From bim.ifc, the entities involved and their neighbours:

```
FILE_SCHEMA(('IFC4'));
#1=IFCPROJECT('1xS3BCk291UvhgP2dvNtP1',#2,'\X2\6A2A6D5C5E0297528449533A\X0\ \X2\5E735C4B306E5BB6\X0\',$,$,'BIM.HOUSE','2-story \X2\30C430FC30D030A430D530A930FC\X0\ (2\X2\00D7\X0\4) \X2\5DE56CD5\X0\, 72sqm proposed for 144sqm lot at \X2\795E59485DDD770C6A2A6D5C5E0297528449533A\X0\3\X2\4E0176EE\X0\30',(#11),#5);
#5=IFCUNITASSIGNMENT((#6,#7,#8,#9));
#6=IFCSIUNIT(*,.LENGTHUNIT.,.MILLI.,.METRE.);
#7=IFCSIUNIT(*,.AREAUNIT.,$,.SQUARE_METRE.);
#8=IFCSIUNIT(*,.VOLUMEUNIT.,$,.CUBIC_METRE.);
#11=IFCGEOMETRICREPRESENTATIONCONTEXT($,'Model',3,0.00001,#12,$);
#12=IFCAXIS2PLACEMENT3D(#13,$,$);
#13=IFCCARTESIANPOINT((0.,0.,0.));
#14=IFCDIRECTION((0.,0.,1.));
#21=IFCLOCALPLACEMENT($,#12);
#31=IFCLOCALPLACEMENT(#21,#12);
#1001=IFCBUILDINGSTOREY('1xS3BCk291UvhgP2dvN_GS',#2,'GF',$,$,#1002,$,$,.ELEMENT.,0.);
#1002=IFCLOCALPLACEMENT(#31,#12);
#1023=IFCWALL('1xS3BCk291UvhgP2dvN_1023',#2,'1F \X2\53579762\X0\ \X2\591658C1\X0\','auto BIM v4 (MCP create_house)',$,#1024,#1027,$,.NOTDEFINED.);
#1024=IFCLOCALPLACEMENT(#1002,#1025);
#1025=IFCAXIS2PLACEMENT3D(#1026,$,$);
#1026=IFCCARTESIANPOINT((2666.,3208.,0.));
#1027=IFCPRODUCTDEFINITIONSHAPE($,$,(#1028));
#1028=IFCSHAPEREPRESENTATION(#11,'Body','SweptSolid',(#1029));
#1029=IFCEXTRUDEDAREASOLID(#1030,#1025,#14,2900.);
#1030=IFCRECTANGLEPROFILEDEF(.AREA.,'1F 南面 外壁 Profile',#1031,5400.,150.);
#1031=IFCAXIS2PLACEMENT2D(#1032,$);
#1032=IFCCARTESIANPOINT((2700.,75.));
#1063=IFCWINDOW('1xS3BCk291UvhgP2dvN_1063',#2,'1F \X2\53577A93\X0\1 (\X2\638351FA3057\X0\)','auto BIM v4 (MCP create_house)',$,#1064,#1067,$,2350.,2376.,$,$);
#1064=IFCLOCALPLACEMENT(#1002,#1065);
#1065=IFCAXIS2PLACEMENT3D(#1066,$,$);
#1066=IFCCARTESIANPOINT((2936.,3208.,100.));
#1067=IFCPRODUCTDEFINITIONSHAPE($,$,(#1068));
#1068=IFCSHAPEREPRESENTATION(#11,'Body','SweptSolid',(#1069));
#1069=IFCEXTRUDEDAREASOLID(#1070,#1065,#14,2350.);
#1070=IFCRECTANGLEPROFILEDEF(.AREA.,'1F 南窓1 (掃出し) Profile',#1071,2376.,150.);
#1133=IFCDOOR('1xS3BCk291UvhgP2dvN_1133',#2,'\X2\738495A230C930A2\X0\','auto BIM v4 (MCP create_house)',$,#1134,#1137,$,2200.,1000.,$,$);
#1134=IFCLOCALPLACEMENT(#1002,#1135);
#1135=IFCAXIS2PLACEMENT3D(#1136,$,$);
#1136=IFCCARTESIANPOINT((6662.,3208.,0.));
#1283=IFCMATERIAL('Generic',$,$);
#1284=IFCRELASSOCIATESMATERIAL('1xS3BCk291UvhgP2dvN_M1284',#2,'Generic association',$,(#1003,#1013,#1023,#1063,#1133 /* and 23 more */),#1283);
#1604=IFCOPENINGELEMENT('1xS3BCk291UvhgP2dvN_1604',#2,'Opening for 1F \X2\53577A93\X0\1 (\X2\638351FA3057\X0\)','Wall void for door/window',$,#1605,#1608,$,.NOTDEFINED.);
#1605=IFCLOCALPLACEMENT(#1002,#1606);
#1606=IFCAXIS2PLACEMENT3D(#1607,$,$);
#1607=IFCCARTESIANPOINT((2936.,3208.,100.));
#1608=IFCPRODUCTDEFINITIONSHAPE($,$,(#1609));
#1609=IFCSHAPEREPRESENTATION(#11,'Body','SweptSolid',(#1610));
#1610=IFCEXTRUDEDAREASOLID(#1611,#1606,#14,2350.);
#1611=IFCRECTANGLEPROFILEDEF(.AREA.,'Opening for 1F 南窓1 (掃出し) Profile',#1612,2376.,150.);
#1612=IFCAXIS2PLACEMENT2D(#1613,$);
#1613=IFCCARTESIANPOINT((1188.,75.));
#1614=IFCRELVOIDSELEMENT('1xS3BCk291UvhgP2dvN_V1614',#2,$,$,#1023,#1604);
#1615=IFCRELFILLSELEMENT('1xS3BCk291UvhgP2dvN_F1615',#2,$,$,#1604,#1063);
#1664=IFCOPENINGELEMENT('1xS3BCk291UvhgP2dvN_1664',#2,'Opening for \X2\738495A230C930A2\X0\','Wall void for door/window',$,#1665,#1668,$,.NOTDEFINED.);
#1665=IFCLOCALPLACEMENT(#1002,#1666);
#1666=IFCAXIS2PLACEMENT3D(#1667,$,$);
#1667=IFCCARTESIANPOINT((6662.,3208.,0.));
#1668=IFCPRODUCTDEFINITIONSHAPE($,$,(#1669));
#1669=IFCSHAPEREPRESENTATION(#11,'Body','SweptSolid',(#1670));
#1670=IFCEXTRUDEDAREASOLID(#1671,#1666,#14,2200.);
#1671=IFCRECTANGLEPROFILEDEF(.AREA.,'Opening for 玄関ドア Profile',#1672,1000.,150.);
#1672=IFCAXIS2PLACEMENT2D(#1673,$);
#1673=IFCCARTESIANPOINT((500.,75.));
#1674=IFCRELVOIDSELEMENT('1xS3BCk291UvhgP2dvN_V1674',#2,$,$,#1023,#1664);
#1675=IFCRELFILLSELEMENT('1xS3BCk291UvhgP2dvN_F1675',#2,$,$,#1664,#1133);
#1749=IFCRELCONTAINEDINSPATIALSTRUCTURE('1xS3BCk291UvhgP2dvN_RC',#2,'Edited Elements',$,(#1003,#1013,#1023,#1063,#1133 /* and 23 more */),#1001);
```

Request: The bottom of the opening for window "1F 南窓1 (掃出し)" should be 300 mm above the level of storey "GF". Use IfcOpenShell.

```python
import numpy as np
import ifcopenshell
import ifcopenshell.api.geometry
import ifcopenshell.geom
import ifcopenshell.util.element
import ifcopenshell.util.placement
import ifcopenshell.util.shape
import ifcopenshell.util.unit

model = ifcopenshell.open("bim.ifc")
unit_scale = ifcopenshell.util.unit.calculate_unit_scale(model)

window = model.by_guid("1xS3BCk291UvhgP2dvN_1063")
opening = window.FillsVoids[0].RelatingOpeningElement
storey = ifcopenshell.util.element.get_container(window, ifc_class="IfcBuildingStorey")
level = ifcopenshell.util.placement.get_local_placement(storey.ObjectPlacement)[2, 3]

# The opening's origin need not be at the sill, so measure its lowest point.
shape = ifcopenshell.geom.create_shape(ifcopenshell.geom.settings(), opening)
bottom = ifcopenshell.util.shape.get_shape_bottom_elevation(shape, shape.geometry) / unit_scale
dz = level + 0.3 / unit_scale - bottom

shift = np.array([0.0, 0.0, dz])
# The window is not placed relative to its opening, so move both.
for product in (opening, window):
    matrix = ifcopenshell.util.placement.get_local_placement(product.ObjectPlacement)
    matrix[:3, 3] += shift
    ifcopenshell.api.geometry.edit_object_placement(model, product=product, matrix=matrix, is_si=False)

print(f"moved by {dz * unit_scale:+.3f} m")

model.write("bim_rev.ifc")
```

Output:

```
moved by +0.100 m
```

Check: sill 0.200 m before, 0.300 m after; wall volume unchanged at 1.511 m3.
